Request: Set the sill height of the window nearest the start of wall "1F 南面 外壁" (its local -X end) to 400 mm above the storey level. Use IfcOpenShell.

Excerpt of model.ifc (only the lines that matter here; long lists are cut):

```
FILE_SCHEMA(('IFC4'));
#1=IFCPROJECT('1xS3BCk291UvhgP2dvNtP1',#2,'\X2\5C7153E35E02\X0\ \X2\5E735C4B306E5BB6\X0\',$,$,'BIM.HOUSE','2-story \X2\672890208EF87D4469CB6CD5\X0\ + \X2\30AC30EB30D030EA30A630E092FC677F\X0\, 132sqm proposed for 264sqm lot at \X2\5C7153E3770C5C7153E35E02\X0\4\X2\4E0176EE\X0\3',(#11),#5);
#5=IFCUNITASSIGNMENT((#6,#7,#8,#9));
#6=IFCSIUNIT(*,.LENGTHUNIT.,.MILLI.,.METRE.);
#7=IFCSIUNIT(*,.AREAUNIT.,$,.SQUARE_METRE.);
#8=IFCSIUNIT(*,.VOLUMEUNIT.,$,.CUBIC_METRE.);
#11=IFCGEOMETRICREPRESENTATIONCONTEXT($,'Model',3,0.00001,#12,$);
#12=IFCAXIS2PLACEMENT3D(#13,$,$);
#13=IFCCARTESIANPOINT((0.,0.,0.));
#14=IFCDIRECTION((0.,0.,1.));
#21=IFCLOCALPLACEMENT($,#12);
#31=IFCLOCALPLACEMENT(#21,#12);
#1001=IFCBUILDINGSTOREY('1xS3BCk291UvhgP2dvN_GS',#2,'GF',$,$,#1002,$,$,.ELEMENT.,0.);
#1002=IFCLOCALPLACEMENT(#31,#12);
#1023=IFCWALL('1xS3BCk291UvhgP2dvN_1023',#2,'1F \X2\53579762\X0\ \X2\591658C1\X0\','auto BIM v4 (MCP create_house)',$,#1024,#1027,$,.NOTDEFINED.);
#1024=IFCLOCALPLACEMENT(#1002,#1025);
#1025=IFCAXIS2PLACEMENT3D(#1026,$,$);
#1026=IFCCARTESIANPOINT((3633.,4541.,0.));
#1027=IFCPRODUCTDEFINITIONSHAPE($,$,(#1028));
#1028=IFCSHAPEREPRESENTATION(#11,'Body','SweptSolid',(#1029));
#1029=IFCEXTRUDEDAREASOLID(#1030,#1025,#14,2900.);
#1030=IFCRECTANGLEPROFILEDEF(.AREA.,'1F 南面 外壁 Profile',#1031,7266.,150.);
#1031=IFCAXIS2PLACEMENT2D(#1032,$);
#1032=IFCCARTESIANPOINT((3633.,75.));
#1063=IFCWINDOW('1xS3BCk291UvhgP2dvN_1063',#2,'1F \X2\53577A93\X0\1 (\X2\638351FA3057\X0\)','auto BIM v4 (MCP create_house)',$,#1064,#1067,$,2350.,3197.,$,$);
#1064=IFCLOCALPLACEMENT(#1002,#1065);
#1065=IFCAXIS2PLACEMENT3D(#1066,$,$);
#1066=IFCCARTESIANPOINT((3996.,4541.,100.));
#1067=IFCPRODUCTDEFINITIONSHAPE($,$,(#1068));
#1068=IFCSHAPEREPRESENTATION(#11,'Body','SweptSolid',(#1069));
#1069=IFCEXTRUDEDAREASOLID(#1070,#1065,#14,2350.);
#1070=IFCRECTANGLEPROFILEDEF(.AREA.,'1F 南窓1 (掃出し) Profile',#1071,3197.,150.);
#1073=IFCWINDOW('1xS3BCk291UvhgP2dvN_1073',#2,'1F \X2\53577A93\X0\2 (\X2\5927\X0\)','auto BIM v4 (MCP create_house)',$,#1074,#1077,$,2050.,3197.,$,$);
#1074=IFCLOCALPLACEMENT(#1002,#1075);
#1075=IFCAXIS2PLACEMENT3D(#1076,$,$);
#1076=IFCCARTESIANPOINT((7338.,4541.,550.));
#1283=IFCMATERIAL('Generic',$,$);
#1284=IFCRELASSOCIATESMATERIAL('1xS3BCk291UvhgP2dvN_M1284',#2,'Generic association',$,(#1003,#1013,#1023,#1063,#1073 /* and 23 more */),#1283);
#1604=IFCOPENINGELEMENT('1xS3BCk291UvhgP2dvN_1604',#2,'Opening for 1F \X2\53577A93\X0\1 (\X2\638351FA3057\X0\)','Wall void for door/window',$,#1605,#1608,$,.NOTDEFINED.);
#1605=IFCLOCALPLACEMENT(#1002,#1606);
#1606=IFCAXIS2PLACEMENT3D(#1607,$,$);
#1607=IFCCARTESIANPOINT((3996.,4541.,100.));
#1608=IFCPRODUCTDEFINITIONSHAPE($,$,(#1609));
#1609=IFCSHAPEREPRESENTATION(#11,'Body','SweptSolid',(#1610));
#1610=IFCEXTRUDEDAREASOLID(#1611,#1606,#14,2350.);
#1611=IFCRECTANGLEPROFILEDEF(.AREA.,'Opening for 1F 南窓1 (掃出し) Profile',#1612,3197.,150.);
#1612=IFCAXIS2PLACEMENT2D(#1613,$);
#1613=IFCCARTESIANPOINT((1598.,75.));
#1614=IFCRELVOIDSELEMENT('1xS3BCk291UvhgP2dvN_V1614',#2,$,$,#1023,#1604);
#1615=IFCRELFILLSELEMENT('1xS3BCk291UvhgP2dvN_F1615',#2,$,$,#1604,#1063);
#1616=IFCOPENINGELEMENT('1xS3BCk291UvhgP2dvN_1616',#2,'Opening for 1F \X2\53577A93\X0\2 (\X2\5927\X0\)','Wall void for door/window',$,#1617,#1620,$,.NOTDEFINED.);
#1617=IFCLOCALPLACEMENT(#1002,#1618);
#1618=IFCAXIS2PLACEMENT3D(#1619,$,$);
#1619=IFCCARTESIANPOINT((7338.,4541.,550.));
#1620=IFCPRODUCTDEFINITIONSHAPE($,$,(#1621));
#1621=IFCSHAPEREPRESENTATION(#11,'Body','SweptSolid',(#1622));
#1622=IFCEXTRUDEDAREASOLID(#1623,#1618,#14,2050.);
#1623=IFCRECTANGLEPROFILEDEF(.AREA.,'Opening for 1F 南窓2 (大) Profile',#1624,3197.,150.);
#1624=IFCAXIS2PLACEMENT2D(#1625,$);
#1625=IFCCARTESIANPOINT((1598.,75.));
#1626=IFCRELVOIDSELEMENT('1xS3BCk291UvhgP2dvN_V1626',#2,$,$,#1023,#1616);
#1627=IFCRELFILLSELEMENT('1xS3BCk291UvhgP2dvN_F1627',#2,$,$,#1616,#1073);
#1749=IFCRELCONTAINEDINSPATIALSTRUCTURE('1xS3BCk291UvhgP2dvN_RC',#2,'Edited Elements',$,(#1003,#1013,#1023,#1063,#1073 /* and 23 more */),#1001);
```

```python
import numpy as np
import ifcopenshell
import ifcopenshell.api.geometry
import ifcopenshell.geom
import ifcopenshell.util.element
import ifcopenshell.util.placement
import ifcopenshell.util.shape
import ifcopenshell.util.unit

model = ifcopenshell.open("model.ifc")
unit_scale = ifcopenshell.util.unit.calculate_unit_scale(model)

window = model.by_guid("1xS3BCk291UvhgP2dvN_1063")
opening = window.FillsVoids[0].RelatingOpeningElement
storey = ifcopenshell.util.element.get_container(window, ifc_class="IfcBuildingStorey")
level = ifcopenshell.util.placement.get_local_placement(storey.ObjectPlacement)[2, 3]

# The opening's origin need not be at the sill, so measure its lowest point.
shape = ifcopenshell.geom.create_shape(ifcopenshell.geom.settings(), opening)
bottom = ifcopenshell.util.shape.get_shape_bottom_elevation(shape, shape.geometry) / unit_scale
dz = level + 0.4 / unit_scale - bottom

shift = np.array([0.0, 0.0, dz])
# The window is not placed relative to its opening, so move both.
for product in (opening, window):
    matrix = ifcopenshell.util.placement.get_local_placement(product.ObjectPlacement)
    matrix[:3, 3] += shift
    ifcopenshell.api.geometry.edit_object_placement(model, product=product, matrix=matrix, is_si=False)

print(f"moved by {dz * unit_scale:+.3f} m")

model.write("model-out.ifc")
```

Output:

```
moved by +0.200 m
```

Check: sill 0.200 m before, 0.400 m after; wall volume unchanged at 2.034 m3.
